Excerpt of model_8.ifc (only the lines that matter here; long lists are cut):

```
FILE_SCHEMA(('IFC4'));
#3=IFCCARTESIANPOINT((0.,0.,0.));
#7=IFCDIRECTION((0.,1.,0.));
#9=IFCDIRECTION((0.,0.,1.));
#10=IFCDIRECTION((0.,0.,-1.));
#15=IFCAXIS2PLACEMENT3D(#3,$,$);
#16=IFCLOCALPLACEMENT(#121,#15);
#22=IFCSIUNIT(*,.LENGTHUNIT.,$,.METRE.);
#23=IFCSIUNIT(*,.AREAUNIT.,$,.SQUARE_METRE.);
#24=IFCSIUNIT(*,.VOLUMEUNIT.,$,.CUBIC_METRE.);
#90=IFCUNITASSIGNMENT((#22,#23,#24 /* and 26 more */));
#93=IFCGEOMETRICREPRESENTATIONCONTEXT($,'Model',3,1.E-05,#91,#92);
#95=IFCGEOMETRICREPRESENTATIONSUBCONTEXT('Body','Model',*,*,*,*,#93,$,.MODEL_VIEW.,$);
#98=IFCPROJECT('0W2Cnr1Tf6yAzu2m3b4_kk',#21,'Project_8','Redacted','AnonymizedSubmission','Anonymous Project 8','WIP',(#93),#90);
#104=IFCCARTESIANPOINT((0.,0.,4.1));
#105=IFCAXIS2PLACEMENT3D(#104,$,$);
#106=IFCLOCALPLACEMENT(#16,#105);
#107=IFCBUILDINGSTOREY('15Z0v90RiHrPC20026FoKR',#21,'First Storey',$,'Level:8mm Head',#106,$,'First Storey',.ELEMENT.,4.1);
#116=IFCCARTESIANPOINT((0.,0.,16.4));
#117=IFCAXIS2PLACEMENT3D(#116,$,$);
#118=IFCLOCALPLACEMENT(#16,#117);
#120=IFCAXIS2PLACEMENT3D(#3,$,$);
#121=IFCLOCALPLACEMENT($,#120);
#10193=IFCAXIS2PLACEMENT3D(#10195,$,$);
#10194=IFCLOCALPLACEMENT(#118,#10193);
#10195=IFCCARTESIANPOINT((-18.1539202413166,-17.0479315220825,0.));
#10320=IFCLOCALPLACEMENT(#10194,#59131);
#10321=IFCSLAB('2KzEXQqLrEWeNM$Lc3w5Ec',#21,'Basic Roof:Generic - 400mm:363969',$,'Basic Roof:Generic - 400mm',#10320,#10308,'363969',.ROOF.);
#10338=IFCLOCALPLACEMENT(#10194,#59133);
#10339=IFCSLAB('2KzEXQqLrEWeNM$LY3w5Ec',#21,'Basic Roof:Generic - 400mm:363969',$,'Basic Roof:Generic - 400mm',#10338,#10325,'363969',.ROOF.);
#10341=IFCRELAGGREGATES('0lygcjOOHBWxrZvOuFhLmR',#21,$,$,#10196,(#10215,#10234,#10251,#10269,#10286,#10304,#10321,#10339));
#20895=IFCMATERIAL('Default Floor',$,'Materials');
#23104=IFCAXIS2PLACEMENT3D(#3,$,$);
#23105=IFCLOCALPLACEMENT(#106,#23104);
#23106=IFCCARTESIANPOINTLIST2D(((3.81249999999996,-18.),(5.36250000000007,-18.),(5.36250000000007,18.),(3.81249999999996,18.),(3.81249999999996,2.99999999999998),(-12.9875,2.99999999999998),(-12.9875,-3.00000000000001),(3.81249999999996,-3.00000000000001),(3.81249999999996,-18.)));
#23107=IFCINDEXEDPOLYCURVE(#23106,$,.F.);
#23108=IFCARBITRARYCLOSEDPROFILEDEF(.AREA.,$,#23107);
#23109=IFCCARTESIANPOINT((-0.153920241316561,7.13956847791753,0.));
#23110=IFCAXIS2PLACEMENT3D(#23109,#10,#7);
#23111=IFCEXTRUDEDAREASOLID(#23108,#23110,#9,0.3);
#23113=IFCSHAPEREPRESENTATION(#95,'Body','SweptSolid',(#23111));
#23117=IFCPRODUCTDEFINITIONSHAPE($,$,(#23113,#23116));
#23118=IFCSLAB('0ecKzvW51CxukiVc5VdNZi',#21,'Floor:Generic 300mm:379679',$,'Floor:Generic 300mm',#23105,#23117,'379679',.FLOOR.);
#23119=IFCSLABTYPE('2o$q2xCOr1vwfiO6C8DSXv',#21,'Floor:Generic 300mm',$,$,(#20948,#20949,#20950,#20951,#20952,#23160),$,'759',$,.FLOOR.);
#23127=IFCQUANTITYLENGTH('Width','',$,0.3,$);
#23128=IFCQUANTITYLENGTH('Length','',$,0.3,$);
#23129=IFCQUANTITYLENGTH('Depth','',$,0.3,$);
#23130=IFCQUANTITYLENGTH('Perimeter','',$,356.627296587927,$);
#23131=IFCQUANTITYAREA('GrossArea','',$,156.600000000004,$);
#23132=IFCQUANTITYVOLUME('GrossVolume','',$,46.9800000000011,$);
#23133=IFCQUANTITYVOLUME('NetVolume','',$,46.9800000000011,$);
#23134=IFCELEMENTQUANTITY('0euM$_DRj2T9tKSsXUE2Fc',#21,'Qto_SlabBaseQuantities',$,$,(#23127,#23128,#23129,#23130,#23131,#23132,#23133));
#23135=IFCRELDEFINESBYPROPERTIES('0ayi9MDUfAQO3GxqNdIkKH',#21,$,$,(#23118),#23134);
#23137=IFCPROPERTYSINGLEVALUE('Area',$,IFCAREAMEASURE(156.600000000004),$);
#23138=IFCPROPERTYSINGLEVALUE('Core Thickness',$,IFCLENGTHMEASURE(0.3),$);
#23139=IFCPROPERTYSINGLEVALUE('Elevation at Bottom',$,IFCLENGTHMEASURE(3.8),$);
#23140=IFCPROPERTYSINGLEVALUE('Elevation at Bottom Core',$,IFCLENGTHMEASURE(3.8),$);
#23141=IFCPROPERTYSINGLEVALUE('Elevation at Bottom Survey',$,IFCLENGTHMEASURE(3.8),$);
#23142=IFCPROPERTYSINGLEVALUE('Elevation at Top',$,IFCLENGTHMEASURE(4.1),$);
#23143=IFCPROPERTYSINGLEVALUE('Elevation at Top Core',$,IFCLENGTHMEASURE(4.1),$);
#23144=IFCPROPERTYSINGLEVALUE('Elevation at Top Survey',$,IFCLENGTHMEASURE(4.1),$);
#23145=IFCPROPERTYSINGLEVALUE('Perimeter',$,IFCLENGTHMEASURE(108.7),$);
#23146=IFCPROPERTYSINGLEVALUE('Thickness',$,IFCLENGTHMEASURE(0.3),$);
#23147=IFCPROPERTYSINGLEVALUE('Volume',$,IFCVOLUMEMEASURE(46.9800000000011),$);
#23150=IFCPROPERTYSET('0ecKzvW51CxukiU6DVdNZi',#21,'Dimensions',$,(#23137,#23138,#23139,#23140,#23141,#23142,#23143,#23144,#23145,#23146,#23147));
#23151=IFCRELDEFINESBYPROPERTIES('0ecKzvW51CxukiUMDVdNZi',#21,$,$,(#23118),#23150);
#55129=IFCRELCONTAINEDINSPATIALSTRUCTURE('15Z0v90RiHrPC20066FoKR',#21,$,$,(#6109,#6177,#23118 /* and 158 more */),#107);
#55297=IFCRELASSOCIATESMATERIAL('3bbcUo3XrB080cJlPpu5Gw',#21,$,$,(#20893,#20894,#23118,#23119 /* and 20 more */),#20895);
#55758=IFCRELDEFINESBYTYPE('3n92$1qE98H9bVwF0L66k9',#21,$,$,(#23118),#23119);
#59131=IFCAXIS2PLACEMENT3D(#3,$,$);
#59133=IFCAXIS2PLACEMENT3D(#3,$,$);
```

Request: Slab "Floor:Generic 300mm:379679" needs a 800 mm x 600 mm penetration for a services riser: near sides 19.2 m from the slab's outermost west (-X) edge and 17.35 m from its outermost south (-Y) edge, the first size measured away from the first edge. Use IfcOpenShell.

```python
import numpy as np
import ifcopenshell
import ifcopenshell.api.feature
import ifcopenshell.api.geometry
import ifcopenshell.api.pset
import ifcopenshell.api.root
import ifcopenshell.geom
import ifcopenshell.util.element
import ifcopenshell.util.placement
import ifcopenshell.util.representation
import ifcopenshell.util.shape
import ifcopenshell.util.unit

model = ifcopenshell.open("model_8.ifc")
unit_scale = ifcopenshell.util.unit.calculate_unit_scale(model)
area_scale = ifcopenshell.util.unit.calculate_unit_scale(model, "AREAUNIT")
volume_scale = ifcopenshell.util.unit.calculate_unit_scale(model, "VOLUMEUNIT")
settings = ifcopenshell.geom.settings()


def volume(element):
    """Net volume in cubic metres, openings subtracted."""
    shape = ifcopenshell.geom.create_shape(settings, element)
    return ifcopenshell.util.shape.get_volume(shape.geometry)


slab = model.by_guid("0ecKzvW51CxukiVc5VdNZi")
before = volume(slab)

# Extent in the slab's own axes, in metres. The edges named are its -X and -Y sides.
slab_shape = ifcopenshell.geom.create_shape(settings, slab)
vertices = ifcopenshell.util.shape.get_vertices(slab_shape.geometry)
x_min, y_min, bottom = vertices.min(axis=0)
top = vertices[:, 2].max()

opening = ifcopenshell.api.root.create_entity(model, ifc_class="IfcOpeningElement", name="Services riser opening", predefined_type="OPENING")
context = ifcopenshell.util.representation.get_context(model, "Model", "Body", "MODEL_VIEW")
width, depth = 0.8, 0.6
outline = [(0.0, 0.0), (width, 0.0), (width, depth), (0.0, depth), (0.0, 0.0)]
# Overshoot both faces by 50 mm so the cut is clean.
shape = ifcopenshell.api.geometry.add_slab_representation(
    model, context=context, depth=top - bottom + 0.1, polyline=outline
)
ifcopenshell.api.geometry.assign_representation(model, product=opening, representation=shape)

matrix = ifcopenshell.util.placement.get_local_placement(slab.ObjectPlacement)
matrix[:, 3] = matrix @ np.append(np.array([x_min + 19.2, y_min + 17.35, bottom - 0.05]) / unit_scale, 1.0)
ifcopenshell.api.geometry.edit_object_placement(model, product=opening, matrix=matrix, is_si=False)
ifcopenshell.api.feature.add_feature(model, feature=opening, element=slab)

after = volume(slab)

# Update the slab's stored quantities.
qto = model.by_id(ifcopenshell.util.element.get_pset(slab, "Qto_SlabBaseQuantities", should_inherit=False)["id"])
ifcopenshell.api.pset.edit_qto(model, qto=qto, properties={"NetVolume": after / volume_scale})
pset = model.by_id(ifcopenshell.util.element.get_pset(slab, "Dimensions", should_inherit=False)["id"])
ifcopenshell.api.pset.edit_pset(model, pset=pset, properties={
    "Area": model.create_entity("IfcAreaMeasure", after / (top - bottom) / area_scale),
    "Volume": model.create_entity("IfcVolumeMeasure", after / volume_scale),
})

print(f"slab volume {before:.3f} -> {after:.3f} m3")

model.write("model_8-out.ifc")
```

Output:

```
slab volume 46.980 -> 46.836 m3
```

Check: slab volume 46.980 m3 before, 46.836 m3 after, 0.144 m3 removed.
